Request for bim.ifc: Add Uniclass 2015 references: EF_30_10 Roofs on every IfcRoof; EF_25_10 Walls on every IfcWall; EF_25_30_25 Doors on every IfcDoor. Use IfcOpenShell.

First a look at what the model holds.

```python
import ifcopenshell

model = ifcopenshell.open("bim.ifc")
print(model.schema)
print("classifications:", [c.Name for c in model.by_type("IfcClassification")])
for ifc_class in ("IfcDoor", "IfcRoof", "IfcStair", "IfcWall", "IfcWindow"):
    print(ifc_class, len(model.by_type(ifc_class)))
```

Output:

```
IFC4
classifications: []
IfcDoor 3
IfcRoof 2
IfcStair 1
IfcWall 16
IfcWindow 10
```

```python
import ifcopenshell
import ifcopenshell.api.classification

model = ifcopenshell.open("bim.ifc")

system = ifcopenshell.api.classification.add_classification(model, classification="Uniclass 2015")

codes = {
    "IfcRoof": ("EF_30_10", "Roofs"),
    "IfcWall": ("EF_25_10", "Walls"),
    "IfcDoor": ("EF_25_30_25", "Doors"),
}
for ifc_class, (code, name) in codes.items():
    products = model.by_type(ifc_class)
    ifcopenshell.api.classification.add_reference(
        model, products=products, classification=system, identification=code, name=name
    )
    print(code, len(products))

model.write("bim_v2.ifc")
```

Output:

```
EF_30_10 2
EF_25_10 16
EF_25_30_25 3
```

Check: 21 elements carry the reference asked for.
